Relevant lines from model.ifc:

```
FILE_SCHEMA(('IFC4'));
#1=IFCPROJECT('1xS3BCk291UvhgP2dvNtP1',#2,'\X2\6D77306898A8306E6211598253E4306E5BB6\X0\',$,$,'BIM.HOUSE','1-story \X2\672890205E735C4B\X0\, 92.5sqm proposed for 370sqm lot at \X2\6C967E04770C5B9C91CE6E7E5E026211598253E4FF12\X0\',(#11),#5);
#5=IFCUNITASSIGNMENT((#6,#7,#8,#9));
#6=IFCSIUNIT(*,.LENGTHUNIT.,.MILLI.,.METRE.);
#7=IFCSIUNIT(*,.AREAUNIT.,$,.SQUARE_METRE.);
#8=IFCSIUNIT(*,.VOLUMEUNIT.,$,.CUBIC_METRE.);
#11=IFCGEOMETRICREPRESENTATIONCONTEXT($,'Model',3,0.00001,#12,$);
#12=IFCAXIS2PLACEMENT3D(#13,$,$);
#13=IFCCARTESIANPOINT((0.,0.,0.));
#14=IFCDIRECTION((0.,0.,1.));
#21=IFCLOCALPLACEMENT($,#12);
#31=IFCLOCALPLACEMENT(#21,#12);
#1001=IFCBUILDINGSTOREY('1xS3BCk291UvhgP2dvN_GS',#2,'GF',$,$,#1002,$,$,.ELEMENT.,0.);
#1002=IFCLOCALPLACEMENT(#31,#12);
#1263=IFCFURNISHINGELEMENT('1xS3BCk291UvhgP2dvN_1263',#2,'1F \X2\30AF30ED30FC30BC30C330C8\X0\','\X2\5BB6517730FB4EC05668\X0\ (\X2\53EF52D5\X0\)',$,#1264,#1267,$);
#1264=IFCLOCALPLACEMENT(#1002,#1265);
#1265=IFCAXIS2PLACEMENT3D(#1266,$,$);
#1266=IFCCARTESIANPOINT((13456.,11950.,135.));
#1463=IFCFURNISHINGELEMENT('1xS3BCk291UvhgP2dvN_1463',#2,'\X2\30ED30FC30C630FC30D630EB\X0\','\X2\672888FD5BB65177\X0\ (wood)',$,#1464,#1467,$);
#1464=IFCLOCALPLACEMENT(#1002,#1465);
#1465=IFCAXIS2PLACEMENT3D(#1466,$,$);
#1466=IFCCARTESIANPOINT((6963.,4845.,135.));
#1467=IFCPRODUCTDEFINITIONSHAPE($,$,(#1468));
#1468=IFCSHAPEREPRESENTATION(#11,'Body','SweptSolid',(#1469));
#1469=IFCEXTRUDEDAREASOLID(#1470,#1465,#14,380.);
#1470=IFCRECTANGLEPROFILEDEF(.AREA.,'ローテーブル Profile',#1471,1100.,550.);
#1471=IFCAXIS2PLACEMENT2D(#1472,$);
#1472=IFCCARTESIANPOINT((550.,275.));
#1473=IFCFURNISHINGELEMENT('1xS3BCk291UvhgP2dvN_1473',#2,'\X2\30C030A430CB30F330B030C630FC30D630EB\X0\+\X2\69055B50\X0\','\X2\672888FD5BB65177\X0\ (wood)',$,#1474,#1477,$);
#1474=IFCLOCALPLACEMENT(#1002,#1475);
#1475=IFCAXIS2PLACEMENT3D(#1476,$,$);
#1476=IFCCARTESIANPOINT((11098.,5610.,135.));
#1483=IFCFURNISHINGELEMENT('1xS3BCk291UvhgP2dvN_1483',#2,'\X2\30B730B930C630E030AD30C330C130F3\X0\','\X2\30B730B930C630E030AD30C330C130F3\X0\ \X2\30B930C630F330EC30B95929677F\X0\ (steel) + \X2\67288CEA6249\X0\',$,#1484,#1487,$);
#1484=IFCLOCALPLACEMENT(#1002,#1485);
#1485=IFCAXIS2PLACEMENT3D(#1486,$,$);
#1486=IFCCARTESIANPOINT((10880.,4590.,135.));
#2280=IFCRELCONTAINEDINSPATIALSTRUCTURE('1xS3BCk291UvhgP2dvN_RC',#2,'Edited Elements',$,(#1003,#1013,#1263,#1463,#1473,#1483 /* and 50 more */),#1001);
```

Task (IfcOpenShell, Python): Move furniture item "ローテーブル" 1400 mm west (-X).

```python
import ifcopenshell
import ifcopenshell.api.geometry
import ifcopenshell.util.placement
import ifcopenshell.util.unit

model = ifcopenshell.open("model.ifc")
unit_scale = ifcopenshell.util.unit.calculate_unit_scale(model)

item = model.by_id(1463)
matrix = ifcopenshell.util.placement.get_local_placement(item.ObjectPlacement)
matrix[0, 3] -= 1.4 / unit_scale
ifcopenshell.api.geometry.edit_object_placement(model, product=item, matrix=matrix, is_si=False)

print(ifcopenshell.util.placement.get_local_placement(item.ObjectPlacement).round(3) + 0.0)

model.write("model-out.ifc")
```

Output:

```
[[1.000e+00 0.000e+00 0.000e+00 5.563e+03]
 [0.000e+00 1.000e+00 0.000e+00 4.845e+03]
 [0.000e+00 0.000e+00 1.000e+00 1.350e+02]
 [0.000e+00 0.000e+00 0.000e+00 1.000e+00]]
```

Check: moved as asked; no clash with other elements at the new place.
